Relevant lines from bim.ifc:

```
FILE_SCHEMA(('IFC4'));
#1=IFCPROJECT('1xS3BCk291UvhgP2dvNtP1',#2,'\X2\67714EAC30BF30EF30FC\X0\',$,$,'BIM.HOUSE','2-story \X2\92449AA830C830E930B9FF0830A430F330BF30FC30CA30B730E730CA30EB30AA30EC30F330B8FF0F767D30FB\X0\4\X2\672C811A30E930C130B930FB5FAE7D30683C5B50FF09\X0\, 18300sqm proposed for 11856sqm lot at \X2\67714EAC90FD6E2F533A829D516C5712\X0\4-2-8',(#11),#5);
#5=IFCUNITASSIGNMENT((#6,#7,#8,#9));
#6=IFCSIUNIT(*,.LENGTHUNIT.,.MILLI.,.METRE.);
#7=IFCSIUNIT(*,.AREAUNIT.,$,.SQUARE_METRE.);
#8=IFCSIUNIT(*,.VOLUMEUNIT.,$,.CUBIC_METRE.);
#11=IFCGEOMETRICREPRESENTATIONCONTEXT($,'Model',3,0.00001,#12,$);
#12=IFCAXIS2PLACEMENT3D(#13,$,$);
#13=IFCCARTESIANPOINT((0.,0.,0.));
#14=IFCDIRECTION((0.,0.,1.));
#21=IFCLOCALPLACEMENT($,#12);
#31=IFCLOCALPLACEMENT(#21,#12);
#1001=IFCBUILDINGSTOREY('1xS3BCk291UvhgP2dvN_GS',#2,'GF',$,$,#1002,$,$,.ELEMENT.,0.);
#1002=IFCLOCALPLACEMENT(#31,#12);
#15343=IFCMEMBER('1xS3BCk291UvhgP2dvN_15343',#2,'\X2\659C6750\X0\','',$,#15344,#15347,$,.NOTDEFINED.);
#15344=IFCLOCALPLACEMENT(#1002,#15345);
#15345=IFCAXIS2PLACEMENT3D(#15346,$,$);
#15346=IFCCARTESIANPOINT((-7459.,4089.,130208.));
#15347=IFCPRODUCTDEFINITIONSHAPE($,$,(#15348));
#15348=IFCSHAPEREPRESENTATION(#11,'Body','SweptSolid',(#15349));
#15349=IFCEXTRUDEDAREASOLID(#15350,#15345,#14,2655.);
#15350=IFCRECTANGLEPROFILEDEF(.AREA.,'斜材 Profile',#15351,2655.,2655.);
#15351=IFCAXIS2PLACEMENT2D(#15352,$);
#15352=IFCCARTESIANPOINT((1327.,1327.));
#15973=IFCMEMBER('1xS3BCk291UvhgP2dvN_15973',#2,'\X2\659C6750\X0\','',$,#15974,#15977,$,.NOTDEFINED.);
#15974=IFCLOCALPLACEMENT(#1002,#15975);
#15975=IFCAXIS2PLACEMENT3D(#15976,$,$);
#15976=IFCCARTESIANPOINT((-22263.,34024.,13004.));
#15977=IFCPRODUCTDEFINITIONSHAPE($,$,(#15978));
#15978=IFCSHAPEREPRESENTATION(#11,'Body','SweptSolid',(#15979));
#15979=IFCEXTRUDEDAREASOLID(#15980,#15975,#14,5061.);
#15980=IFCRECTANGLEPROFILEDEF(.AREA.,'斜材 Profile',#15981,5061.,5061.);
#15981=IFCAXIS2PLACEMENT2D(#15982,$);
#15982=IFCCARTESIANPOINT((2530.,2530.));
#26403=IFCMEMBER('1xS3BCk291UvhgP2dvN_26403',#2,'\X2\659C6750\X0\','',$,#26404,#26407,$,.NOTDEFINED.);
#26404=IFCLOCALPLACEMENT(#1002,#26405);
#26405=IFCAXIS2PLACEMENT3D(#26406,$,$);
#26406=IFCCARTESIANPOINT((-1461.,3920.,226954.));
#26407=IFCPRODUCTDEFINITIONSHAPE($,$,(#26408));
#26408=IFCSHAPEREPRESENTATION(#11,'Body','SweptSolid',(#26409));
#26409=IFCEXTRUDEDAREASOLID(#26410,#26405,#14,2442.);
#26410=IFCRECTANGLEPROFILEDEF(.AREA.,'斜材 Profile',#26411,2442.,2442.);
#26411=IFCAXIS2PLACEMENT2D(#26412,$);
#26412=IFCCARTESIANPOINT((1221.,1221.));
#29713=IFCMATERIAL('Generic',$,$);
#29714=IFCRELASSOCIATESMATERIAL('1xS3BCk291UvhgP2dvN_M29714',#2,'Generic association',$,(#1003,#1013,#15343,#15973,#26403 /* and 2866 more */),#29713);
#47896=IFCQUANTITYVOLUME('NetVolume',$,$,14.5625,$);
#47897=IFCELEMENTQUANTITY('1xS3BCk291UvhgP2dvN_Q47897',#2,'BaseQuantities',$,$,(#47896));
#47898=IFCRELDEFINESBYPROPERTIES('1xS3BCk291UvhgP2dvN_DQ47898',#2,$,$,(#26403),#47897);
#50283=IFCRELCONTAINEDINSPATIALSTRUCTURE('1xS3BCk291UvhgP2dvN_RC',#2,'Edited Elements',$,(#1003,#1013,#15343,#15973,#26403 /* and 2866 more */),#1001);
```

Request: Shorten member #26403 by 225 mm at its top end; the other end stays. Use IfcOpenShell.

```python
import ifcopenshell
import ifcopenshell.api.pset
import ifcopenshell.util.element

model = ifcopenshell.open("bim.ifc")

member = model.by_guid("1xS3BCk291UvhgP2dvN_26403")
change = -225.0

# The extrusion runs towards the end named, so only its depth changes.
body = next(r for r in member.Representation.Representations if r.RepresentationIdentifier == "Body")
solid = body.Items[0]
old_length = solid.Depth
solid.Depth += change

# Update the stored length and volume.
qto = model.by_id(ifcopenshell.util.element.get_pset(member, "BaseQuantities", should_inherit=False)["id"])
ifcopenshell.api.pset.edit_qto(model, qto=qto, properties={
    "NetVolume": ifcopenshell.util.element.get_pset(member, "BaseQuantities", "NetVolume") * solid.Depth / old_length,
})

print(f"length {old_length:g} -> {solid.Depth:g}")

model.write("bim-out.ifc")
```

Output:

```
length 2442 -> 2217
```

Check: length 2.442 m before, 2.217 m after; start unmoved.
